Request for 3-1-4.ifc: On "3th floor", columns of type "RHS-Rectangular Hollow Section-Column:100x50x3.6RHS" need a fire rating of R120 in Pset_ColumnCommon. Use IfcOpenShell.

First a look at what the model holds.

```python
import ifcopenshell
import ifcopenshell.util.element

model = ifcopenshell.open("3-1-4.ifc")
print(model.schema)
storey = next(s for s in model.by_type("IfcBuildingStorey") if s.Name == "3th floor")
columns = [e for e in ifcopenshell.util.element.get_decomposition(storey) if e.is_a("IfcColumn")]
seen = {}
for e in columns:
    element_type = ifcopenshell.util.element.get_type(e)
    key = (element_type.Name if element_type != e and element_type else None, ifcopenshell.util.element.get_pset(e, "Pset_ColumnCommon", "FireRating"))
    seen[key] = seen.get(key, 0) + 1
for (name, value), count in sorted(seen.items(), key=str):
    print(count, "x", name, "|", value)
```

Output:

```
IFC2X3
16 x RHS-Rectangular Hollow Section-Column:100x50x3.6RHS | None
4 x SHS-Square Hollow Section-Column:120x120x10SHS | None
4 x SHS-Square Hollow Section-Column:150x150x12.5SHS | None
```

```python
import ifcopenshell
import ifcopenshell.api.pset
import ifcopenshell.util.element

model = ifcopenshell.open("3-1-4.ifc")

storey = next(s for s in model.by_type("IfcBuildingStorey") if s.Name == "3th floor")
columns = [e for e in ifcopenshell.util.element.get_decomposition(storey) if e.is_a("IfcColumn")]

count = 0
for e in columns:
    element_type = ifcopenshell.util.element.get_type(e)
    if element_type in (None, e) or element_type.Name != "RHS-Rectangular Hollow Section-Column:100x50x3.6RHS":
        continue
    # add_pset returns the element's existing set when there is one.
    pset = ifcopenshell.api.pset.add_pset(model, product=e, name="Pset_ColumnCommon")
    ifcopenshell.api.pset.edit_pset(model, pset=pset, properties={"FireRating": "R120"})
    count += 1

print(count, "columns updated")

model.write("3-1-4_rev.ifc")
```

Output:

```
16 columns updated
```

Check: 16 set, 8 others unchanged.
